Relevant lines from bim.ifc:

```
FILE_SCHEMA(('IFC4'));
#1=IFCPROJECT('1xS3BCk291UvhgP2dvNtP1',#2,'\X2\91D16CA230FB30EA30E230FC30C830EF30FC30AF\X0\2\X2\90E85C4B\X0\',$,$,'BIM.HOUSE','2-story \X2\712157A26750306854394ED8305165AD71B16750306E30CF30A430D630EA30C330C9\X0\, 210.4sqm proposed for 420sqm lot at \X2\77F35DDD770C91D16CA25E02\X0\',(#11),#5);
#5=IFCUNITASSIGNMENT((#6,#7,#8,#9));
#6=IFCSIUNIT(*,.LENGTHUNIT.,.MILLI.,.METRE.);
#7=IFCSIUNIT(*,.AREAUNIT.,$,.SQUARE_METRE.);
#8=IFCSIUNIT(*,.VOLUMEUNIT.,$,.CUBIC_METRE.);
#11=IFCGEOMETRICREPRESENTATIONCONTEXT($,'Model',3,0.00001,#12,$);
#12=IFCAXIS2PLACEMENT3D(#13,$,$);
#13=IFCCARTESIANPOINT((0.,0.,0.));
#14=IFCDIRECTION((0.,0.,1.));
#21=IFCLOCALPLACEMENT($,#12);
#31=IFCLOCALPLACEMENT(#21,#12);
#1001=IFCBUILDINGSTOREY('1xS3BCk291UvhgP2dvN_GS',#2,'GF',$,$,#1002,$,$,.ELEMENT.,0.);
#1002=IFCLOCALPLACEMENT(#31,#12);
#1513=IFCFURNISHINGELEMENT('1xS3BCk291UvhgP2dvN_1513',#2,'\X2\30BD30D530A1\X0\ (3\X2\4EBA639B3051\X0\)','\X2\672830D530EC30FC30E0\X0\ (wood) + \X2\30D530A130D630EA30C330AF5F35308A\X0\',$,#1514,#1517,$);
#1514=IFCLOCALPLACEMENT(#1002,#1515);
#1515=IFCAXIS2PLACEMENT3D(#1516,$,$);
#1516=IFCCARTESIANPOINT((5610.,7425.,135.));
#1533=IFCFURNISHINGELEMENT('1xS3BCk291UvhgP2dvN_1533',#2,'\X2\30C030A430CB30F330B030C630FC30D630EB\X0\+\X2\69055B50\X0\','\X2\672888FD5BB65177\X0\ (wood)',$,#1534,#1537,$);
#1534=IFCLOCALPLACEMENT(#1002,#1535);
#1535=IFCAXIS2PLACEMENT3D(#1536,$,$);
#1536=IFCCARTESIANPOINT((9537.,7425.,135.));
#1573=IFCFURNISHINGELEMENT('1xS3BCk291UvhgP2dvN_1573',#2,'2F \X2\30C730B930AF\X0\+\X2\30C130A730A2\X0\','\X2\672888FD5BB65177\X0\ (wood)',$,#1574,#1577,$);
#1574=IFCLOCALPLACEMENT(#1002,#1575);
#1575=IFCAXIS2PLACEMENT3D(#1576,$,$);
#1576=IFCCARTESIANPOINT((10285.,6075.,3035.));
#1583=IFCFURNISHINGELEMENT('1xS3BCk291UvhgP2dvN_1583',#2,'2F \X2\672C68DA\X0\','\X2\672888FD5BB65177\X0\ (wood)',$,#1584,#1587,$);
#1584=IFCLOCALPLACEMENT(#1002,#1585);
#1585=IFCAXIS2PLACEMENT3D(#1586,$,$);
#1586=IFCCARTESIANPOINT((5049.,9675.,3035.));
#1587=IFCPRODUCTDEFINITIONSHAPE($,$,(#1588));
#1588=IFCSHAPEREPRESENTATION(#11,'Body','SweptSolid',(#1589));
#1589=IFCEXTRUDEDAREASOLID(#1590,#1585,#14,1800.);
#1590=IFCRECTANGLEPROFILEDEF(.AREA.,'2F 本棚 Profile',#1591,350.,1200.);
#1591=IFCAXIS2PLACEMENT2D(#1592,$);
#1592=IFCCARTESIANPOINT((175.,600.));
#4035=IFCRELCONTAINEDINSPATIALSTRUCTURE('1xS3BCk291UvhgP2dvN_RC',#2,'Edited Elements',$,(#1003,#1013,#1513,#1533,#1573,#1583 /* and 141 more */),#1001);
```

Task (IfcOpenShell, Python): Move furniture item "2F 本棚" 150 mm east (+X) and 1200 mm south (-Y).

```python
import ifcopenshell
import ifcopenshell.api.geometry
import ifcopenshell.util.placement
import ifcopenshell.util.unit

model = ifcopenshell.open("bim.ifc")
unit_scale = ifcopenshell.util.unit.calculate_unit_scale(model)

item = model.by_guid("1xS3BCk291UvhgP2dvN_1583")
matrix = ifcopenshell.util.placement.get_local_placement(item.ObjectPlacement)
matrix[0, 3] += 0.15 / unit_scale
matrix[1, 3] -= 1.2 / unit_scale
ifcopenshell.api.geometry.edit_object_placement(model, product=item, matrix=matrix, is_si=False)

print(ifcopenshell.util.placement.get_local_placement(item.ObjectPlacement).round(3) + 0.0)

model.write("bim_updated.ifc")
```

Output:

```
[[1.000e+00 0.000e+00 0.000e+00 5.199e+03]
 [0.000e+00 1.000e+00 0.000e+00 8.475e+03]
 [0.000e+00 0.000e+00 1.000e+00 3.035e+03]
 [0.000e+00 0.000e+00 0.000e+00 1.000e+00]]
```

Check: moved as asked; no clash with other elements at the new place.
